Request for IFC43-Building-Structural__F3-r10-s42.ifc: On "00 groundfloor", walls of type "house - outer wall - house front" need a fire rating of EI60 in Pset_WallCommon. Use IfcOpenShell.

First a look at what the model holds.

```python
import ifcopenshell
import ifcopenshell.util.element

model = ifcopenshell.open("IFC43-Building-Structural__F3-r10-s42.ifc")
print(model.schema)
storey = next(s for s in model.by_type("IfcBuildingStorey") if s.Name == "00 groundfloor")
walls = [e for e in ifcopenshell.util.element.get_decomposition(storey) if e.is_a("IfcWall")]
seen = {}
for e in walls:
    element_type = ifcopenshell.util.element.get_type(e)
    key = (element_type.Name if element_type != e and element_type else None, ifcopenshell.util.element.get_pset(e, "Pset_WallCommon", "FireRating"))
    seen[key] = seen.get(key, 0) + 1
for (name, value), count in sorted(seen.items(), key=str):
    print(count, "x", name, "|", value)
```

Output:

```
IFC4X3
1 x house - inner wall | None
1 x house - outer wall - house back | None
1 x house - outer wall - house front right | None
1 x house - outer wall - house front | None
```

```python
import ifcopenshell
import ifcopenshell.api.pset
import ifcopenshell.util.element

model = ifcopenshell.open("IFC43-Building-Structural__F3-r10-s42.ifc")

storey = next(s for s in model.by_type("IfcBuildingStorey") if s.Name == "00 groundfloor")
walls = [e for e in ifcopenshell.util.element.get_decomposition(storey) if e.is_a("IfcWall")]

count = 0
for e in walls:
    element_type = ifcopenshell.util.element.get_type(e)
    if element_type in (None, e) or element_type.Name != "house - outer wall - house front":
        continue
    # add_pset returns the element's existing set when there is one.
    pset = ifcopenshell.api.pset.add_pset(model, product=e, name="Pset_WallCommon")
    ifcopenshell.api.pset.edit_pset(model, pset=pset, properties={"FireRating": "EI60"})
    count += 1

print(count, "walls updated")

model.write("IFC43-Building-Structural__F3-r10-s42_updated.ifc")
```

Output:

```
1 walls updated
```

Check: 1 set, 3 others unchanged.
